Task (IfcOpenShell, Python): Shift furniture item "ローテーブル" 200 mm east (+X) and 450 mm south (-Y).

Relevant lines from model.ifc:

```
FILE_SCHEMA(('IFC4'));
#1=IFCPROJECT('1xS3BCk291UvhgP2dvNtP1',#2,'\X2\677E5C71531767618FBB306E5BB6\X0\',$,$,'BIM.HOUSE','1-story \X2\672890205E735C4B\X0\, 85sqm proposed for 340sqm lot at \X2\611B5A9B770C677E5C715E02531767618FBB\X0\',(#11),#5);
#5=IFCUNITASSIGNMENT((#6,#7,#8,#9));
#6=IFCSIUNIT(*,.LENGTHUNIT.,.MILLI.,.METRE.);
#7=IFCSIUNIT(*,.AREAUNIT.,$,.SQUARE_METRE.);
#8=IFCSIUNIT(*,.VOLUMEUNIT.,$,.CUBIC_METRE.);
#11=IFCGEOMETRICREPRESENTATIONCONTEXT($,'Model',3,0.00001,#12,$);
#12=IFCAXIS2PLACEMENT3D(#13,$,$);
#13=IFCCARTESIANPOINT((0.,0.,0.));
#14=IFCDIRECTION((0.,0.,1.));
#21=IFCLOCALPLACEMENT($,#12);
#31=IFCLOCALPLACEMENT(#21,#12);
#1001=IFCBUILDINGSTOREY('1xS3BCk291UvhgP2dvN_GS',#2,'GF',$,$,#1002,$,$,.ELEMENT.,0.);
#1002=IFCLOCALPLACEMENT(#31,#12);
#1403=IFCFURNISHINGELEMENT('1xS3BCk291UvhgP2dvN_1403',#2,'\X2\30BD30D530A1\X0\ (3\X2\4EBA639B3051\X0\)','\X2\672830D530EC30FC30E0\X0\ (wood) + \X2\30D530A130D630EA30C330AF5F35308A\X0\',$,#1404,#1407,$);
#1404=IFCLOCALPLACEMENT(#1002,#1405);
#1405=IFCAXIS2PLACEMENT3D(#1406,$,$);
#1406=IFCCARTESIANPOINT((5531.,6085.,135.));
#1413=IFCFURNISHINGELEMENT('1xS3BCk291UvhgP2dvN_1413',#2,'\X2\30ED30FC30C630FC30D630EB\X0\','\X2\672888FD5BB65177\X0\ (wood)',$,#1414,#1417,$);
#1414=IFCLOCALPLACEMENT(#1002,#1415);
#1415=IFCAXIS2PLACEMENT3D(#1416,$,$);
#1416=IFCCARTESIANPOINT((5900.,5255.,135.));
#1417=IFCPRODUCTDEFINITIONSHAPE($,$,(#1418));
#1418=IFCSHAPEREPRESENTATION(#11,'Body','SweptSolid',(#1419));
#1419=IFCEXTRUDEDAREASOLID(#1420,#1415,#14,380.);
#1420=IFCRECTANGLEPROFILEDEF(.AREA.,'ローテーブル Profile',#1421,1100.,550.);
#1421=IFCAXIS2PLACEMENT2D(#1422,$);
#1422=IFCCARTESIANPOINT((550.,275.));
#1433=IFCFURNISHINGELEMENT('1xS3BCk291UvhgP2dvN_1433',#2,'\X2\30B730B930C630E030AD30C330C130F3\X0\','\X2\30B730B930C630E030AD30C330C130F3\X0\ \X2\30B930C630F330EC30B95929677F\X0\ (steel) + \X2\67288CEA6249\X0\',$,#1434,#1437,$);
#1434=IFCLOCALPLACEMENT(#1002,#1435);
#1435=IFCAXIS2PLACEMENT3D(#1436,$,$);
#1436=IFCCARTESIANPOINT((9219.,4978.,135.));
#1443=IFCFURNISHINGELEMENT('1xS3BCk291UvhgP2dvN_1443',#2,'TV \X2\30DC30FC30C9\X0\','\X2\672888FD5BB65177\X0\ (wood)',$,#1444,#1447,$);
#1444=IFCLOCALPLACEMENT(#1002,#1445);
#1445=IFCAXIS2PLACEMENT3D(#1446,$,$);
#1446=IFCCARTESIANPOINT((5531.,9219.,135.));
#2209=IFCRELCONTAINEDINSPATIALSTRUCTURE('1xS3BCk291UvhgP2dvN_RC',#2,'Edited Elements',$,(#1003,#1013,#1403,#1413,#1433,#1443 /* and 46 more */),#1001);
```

```python
import ifcopenshell
import ifcopenshell.api.geometry
import ifcopenshell.util.placement

model = ifcopenshell.open("model.ifc")

item = model.by_guid("1xS3BCk291UvhgP2dvN_1413")
matrix = ifcopenshell.util.placement.get_local_placement(item.ObjectPlacement)
matrix[0, 3] += 200.0
matrix[1, 3] -= 450.0
ifcopenshell.api.geometry.edit_object_placement(model, product=item, matrix=matrix, is_si=False)

print(ifcopenshell.util.placement.get_local_placement(item.ObjectPlacement).round(3) + 0.0)

model.write("model_v2.ifc")
```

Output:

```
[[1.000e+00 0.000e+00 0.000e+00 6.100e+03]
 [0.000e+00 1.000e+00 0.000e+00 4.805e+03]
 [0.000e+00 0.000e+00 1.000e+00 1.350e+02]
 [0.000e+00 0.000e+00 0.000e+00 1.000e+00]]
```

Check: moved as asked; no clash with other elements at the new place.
